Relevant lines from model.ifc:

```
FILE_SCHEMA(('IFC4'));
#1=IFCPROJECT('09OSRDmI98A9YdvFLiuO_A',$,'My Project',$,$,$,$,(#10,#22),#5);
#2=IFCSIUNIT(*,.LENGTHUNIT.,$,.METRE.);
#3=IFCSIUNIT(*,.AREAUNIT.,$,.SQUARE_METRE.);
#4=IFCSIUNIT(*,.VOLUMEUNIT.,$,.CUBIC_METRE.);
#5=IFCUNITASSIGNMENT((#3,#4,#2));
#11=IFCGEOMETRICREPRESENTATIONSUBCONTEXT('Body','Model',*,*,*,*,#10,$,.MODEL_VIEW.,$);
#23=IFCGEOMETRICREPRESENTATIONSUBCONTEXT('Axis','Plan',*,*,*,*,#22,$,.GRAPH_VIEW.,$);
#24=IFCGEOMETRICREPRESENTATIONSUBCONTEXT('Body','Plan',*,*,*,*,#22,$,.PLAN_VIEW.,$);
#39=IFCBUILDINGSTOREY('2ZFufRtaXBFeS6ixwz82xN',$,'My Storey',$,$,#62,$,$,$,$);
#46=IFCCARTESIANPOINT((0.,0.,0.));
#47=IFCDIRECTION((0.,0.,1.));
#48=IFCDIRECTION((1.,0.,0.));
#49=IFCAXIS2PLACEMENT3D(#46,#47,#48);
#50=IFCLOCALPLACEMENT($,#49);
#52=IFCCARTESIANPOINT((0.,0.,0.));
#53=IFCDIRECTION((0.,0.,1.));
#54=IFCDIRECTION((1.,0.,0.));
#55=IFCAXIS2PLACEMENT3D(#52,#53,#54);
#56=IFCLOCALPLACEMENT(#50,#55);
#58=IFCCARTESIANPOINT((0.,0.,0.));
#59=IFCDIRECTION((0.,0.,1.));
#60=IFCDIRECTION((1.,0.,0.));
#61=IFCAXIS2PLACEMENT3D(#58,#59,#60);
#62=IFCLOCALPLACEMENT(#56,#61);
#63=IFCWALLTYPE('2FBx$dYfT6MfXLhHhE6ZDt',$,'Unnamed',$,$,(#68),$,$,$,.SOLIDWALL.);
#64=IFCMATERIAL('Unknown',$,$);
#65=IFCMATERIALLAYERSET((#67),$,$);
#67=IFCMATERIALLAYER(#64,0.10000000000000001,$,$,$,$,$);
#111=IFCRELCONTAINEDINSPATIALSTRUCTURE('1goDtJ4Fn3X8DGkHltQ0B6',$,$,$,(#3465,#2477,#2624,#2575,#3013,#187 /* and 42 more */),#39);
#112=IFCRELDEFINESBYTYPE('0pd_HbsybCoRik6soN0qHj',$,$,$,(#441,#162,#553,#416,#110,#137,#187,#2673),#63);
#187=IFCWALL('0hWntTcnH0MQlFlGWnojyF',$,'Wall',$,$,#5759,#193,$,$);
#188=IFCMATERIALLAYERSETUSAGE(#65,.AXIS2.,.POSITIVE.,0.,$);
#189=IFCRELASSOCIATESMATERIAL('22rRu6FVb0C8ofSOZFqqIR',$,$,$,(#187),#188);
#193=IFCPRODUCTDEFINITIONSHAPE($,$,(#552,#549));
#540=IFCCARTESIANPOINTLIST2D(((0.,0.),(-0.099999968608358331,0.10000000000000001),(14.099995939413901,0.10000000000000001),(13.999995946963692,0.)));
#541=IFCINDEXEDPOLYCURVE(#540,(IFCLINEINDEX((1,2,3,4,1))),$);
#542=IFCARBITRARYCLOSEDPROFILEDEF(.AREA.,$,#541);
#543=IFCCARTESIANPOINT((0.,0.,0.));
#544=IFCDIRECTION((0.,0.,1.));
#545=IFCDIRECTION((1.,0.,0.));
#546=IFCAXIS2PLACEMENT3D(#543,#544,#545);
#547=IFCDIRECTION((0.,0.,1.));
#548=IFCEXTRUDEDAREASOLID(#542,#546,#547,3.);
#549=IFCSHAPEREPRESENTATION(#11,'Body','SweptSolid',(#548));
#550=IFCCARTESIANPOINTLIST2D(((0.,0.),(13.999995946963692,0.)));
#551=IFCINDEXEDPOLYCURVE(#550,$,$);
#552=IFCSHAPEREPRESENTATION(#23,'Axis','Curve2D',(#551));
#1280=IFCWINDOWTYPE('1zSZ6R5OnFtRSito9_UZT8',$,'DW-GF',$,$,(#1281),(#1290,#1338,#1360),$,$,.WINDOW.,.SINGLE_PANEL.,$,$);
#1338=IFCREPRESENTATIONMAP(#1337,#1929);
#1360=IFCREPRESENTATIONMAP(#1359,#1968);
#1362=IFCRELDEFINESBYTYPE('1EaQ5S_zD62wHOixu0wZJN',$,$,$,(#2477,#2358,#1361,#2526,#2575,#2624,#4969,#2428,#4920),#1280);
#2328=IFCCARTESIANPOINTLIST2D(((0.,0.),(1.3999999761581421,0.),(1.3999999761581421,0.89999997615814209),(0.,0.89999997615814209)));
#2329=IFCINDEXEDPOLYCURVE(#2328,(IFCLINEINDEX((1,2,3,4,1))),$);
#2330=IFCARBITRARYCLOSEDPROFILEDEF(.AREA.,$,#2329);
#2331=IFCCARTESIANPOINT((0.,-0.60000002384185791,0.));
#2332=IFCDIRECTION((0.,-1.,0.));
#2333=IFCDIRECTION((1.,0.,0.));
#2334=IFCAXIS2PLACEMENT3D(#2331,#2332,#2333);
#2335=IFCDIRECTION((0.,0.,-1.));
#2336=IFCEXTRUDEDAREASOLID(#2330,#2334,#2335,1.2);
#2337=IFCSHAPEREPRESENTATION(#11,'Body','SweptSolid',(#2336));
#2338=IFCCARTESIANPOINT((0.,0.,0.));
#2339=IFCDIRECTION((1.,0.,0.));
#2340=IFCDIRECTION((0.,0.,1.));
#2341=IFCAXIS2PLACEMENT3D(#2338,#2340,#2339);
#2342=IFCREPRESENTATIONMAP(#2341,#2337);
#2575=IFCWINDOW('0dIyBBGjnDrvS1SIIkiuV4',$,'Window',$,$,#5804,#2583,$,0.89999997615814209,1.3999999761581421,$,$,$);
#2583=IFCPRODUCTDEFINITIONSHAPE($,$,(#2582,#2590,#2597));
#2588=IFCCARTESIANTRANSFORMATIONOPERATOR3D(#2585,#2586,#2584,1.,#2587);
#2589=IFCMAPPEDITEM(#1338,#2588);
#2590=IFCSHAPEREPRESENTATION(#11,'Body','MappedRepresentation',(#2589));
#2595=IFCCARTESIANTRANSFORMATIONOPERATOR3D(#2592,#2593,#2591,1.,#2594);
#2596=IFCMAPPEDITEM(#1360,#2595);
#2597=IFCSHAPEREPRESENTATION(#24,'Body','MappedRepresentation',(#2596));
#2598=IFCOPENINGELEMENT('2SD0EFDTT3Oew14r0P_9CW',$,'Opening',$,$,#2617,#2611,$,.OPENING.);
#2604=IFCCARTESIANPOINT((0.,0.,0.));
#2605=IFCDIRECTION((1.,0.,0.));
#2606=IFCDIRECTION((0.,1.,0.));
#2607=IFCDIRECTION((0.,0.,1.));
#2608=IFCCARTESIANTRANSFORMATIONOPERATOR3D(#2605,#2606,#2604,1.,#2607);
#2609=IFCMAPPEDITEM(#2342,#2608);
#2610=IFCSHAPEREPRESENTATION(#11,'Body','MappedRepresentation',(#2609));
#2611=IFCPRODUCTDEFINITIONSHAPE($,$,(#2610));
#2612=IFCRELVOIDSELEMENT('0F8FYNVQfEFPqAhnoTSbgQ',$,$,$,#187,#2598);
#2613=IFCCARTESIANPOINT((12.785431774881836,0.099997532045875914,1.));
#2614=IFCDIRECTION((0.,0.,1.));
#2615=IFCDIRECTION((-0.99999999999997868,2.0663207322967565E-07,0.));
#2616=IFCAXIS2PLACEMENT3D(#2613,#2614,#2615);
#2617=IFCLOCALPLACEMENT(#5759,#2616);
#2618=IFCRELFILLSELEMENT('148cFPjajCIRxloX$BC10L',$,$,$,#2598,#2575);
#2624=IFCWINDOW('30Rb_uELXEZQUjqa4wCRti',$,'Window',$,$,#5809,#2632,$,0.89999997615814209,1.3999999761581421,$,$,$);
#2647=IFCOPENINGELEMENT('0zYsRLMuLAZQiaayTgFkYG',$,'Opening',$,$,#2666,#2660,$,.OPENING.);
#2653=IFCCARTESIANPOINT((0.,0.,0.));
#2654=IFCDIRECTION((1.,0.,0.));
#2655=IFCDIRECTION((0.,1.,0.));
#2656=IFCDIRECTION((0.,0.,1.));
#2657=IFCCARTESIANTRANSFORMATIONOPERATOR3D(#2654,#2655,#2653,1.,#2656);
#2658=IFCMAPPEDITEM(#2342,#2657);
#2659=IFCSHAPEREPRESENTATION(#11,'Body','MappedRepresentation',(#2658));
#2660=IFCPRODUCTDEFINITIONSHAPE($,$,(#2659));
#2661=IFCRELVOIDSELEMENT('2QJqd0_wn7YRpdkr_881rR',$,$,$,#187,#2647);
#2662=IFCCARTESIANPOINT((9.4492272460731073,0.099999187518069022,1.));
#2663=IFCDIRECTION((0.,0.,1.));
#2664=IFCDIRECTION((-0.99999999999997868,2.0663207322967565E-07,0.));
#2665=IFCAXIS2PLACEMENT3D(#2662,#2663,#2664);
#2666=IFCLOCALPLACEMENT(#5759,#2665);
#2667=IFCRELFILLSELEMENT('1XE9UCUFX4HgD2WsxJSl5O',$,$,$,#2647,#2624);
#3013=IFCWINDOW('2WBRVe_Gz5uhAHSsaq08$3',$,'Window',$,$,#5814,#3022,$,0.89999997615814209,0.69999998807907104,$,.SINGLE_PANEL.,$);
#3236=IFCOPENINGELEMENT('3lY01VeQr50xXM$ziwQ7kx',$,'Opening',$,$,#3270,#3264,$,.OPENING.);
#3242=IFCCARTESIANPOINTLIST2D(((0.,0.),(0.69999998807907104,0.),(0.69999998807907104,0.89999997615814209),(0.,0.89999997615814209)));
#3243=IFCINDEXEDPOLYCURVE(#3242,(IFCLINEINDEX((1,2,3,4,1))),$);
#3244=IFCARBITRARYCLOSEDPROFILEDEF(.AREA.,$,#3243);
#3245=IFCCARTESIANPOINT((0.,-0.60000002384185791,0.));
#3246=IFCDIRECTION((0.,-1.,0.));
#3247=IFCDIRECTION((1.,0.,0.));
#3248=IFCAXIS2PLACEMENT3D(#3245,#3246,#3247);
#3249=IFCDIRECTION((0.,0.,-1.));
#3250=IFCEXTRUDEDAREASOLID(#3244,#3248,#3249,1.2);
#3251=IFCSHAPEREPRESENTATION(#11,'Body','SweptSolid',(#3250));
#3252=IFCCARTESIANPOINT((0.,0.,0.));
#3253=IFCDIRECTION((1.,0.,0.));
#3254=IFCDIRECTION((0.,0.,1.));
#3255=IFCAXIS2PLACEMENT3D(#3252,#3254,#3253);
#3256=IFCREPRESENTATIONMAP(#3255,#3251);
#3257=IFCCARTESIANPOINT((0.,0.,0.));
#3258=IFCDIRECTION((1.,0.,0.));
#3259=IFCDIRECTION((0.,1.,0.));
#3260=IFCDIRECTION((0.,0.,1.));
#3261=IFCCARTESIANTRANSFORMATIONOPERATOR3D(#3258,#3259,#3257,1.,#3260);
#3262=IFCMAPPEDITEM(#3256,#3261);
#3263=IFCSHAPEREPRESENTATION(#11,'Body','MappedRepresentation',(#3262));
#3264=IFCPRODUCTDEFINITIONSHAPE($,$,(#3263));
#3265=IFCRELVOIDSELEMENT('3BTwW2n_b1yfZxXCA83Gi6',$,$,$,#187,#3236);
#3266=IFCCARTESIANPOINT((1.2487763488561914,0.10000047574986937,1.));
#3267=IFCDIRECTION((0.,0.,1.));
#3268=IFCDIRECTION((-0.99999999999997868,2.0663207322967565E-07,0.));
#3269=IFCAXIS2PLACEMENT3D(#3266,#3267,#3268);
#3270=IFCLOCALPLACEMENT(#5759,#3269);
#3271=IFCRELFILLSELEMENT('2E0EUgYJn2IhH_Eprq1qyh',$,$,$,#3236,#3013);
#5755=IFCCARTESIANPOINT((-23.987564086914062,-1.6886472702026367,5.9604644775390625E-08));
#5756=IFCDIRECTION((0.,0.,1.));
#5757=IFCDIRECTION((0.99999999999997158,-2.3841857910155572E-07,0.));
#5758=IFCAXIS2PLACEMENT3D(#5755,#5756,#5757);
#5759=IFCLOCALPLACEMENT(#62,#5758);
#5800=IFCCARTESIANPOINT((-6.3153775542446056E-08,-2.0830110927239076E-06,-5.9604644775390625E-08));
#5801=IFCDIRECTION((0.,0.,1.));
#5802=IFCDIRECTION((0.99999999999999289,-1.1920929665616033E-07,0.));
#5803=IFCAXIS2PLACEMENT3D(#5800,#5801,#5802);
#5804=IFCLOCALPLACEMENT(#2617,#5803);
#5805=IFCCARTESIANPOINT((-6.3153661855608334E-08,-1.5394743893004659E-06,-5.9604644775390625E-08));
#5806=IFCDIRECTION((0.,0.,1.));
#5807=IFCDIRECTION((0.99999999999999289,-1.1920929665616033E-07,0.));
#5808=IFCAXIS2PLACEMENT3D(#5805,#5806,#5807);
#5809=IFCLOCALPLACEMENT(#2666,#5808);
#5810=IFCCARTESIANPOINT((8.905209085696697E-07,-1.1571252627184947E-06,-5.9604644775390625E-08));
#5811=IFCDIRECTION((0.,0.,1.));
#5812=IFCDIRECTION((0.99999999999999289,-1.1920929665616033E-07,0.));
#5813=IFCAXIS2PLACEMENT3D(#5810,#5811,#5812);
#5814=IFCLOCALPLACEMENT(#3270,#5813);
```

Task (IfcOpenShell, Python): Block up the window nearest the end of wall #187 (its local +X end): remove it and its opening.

```python
import ifcopenshell
import ifcopenshell.api.feature
import ifcopenshell.api.root
import ifcopenshell.geom
import ifcopenshell.util.shape

model = ifcopenshell.open("model.ifc")
settings = ifcopenshell.geom.settings()


def volume(element):
    """Net volume in cubic metres, openings subtracted."""
    shape = ifcopenshell.geom.create_shape(settings, element)
    return ifcopenshell.util.shape.get_volume(shape.geometry)


window = model.by_id(2575)
opening = window.FillsVoids[0].RelatingOpeningElement
wall = opening.VoidsElements[0].RelatingBuildingElement
before = volume(wall)

ifcopenshell.api.root.remove_product(model, product=window)
ifcopenshell.api.feature.remove_feature(model, feature=opening)

after = volume(wall)

print(f"wall volume {before:.3f} -> {after:.3f} m3")

model.write("model_v2.ifc")
```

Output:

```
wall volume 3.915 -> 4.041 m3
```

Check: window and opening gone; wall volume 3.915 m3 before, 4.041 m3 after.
